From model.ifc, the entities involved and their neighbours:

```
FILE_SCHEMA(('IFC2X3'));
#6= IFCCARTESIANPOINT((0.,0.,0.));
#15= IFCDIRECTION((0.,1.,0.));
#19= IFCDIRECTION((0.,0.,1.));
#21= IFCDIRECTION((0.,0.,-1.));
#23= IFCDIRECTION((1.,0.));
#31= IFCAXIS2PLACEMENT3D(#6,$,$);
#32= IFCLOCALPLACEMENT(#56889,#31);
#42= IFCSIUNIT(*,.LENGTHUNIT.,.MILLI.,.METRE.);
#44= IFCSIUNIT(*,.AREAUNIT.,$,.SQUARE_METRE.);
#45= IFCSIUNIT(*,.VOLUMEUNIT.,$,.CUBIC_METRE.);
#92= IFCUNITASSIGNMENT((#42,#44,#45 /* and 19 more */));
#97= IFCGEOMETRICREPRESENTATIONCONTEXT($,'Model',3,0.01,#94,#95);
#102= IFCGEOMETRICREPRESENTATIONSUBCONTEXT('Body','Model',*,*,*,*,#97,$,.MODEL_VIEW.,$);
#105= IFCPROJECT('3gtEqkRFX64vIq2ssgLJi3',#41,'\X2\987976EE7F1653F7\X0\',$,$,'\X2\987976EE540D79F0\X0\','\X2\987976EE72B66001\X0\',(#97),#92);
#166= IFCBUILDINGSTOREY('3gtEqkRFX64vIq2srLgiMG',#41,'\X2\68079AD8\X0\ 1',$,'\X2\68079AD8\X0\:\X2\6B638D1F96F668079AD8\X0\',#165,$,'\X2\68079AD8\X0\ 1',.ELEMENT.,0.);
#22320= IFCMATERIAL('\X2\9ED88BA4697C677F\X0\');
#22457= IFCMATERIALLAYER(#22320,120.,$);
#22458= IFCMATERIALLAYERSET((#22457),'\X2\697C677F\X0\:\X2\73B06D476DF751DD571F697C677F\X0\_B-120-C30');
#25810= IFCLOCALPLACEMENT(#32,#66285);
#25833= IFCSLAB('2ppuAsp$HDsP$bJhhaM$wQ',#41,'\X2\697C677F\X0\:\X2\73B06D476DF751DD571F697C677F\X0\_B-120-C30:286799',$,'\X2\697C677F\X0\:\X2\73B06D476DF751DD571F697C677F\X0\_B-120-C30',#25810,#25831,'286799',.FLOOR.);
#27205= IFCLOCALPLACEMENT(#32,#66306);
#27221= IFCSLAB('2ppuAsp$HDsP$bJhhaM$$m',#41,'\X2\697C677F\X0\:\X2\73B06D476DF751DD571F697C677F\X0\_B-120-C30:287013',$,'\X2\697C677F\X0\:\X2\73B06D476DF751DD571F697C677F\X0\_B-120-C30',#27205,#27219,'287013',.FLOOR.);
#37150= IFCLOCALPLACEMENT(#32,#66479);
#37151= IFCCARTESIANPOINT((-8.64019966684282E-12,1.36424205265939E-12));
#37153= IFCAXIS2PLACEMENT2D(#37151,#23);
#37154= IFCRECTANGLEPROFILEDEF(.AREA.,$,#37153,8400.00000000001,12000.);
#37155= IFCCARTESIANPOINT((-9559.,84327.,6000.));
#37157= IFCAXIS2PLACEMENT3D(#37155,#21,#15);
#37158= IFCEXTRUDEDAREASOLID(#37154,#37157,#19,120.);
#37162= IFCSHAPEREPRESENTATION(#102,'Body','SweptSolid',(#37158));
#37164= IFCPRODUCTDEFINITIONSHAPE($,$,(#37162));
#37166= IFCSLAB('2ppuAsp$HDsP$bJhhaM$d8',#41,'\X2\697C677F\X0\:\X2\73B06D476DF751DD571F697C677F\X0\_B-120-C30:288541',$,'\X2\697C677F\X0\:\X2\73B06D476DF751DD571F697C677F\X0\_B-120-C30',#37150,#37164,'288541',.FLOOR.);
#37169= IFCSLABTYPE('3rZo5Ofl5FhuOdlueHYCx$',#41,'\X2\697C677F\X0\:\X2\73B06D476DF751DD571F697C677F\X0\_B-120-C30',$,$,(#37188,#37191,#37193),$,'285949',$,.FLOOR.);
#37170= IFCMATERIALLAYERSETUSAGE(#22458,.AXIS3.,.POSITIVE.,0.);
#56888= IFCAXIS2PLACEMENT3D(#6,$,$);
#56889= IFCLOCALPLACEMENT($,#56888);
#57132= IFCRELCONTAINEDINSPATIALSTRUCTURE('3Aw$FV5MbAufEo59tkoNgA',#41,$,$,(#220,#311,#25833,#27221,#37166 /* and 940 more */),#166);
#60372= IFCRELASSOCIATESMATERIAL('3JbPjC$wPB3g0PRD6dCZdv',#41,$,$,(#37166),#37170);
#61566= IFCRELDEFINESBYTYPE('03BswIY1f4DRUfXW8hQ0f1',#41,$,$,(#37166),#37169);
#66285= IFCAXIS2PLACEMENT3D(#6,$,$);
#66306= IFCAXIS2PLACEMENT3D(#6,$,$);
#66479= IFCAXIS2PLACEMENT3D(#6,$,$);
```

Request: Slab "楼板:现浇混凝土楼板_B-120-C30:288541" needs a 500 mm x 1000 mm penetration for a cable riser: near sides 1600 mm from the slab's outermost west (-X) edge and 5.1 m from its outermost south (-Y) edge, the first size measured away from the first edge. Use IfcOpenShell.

```python
import numpy as np
import ifcopenshell
import ifcopenshell.api.feature
import ifcopenshell.api.geometry
import ifcopenshell.api.root
import ifcopenshell.geom
import ifcopenshell.util.placement
import ifcopenshell.util.representation
import ifcopenshell.util.shape
import ifcopenshell.util.unit

model = ifcopenshell.open("model.ifc")
unit_scale = ifcopenshell.util.unit.calculate_unit_scale(model)
settings = ifcopenshell.geom.settings()


def volume(element):
    """Net volume in cubic metres, openings subtracted."""
    shape = ifcopenshell.geom.create_shape(settings, element)
    return ifcopenshell.util.shape.get_volume(shape.geometry)


slab = model.by_guid("2ppuAsp$HDsP$bJhhaM$d8")
before = volume(slab)

# Extent in the slab's own axes, in metres. The edges named are its -X and -Y sides.
slab_shape = ifcopenshell.geom.create_shape(settings, slab)
vertices = ifcopenshell.util.shape.get_vertices(slab_shape.geometry)
x_min, y_min, bottom = vertices.min(axis=0)
top = vertices[:, 2].max()

opening = ifcopenshell.api.root.create_entity(model, ifc_class="IfcOpeningElement", name="Cable riser opening")
context = ifcopenshell.util.representation.get_context(model, "Model", "Body", "MODEL_VIEW")
width, depth = 0.5, 1
outline = [(0.0, 0.0), (width, 0.0), (width, depth), (0.0, depth), (0.0, 0.0)]
# Overshoot both faces by 50 mm so the cut is clean.
shape = ifcopenshell.api.geometry.add_slab_representation(
    model, context=context, depth=top - bottom + 0.1, polyline=outline
)
ifcopenshell.api.geometry.assign_representation(model, product=opening, representation=shape)

matrix = ifcopenshell.util.placement.get_local_placement(slab.ObjectPlacement)
matrix[:, 3] = matrix @ np.append(np.array([x_min + 1.6, y_min + 5.1, bottom - 0.05]) / unit_scale, 1.0)
ifcopenshell.api.geometry.edit_object_placement(model, product=opening, matrix=matrix, is_si=False)
ifcopenshell.api.feature.add_feature(model, feature=opening, element=slab)

after = volume(slab)

print(f"slab volume {before:.3f} -> {after:.3f} m3")

model.write("model_rev.ifc")
```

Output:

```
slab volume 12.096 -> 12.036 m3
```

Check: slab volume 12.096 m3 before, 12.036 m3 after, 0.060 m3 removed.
